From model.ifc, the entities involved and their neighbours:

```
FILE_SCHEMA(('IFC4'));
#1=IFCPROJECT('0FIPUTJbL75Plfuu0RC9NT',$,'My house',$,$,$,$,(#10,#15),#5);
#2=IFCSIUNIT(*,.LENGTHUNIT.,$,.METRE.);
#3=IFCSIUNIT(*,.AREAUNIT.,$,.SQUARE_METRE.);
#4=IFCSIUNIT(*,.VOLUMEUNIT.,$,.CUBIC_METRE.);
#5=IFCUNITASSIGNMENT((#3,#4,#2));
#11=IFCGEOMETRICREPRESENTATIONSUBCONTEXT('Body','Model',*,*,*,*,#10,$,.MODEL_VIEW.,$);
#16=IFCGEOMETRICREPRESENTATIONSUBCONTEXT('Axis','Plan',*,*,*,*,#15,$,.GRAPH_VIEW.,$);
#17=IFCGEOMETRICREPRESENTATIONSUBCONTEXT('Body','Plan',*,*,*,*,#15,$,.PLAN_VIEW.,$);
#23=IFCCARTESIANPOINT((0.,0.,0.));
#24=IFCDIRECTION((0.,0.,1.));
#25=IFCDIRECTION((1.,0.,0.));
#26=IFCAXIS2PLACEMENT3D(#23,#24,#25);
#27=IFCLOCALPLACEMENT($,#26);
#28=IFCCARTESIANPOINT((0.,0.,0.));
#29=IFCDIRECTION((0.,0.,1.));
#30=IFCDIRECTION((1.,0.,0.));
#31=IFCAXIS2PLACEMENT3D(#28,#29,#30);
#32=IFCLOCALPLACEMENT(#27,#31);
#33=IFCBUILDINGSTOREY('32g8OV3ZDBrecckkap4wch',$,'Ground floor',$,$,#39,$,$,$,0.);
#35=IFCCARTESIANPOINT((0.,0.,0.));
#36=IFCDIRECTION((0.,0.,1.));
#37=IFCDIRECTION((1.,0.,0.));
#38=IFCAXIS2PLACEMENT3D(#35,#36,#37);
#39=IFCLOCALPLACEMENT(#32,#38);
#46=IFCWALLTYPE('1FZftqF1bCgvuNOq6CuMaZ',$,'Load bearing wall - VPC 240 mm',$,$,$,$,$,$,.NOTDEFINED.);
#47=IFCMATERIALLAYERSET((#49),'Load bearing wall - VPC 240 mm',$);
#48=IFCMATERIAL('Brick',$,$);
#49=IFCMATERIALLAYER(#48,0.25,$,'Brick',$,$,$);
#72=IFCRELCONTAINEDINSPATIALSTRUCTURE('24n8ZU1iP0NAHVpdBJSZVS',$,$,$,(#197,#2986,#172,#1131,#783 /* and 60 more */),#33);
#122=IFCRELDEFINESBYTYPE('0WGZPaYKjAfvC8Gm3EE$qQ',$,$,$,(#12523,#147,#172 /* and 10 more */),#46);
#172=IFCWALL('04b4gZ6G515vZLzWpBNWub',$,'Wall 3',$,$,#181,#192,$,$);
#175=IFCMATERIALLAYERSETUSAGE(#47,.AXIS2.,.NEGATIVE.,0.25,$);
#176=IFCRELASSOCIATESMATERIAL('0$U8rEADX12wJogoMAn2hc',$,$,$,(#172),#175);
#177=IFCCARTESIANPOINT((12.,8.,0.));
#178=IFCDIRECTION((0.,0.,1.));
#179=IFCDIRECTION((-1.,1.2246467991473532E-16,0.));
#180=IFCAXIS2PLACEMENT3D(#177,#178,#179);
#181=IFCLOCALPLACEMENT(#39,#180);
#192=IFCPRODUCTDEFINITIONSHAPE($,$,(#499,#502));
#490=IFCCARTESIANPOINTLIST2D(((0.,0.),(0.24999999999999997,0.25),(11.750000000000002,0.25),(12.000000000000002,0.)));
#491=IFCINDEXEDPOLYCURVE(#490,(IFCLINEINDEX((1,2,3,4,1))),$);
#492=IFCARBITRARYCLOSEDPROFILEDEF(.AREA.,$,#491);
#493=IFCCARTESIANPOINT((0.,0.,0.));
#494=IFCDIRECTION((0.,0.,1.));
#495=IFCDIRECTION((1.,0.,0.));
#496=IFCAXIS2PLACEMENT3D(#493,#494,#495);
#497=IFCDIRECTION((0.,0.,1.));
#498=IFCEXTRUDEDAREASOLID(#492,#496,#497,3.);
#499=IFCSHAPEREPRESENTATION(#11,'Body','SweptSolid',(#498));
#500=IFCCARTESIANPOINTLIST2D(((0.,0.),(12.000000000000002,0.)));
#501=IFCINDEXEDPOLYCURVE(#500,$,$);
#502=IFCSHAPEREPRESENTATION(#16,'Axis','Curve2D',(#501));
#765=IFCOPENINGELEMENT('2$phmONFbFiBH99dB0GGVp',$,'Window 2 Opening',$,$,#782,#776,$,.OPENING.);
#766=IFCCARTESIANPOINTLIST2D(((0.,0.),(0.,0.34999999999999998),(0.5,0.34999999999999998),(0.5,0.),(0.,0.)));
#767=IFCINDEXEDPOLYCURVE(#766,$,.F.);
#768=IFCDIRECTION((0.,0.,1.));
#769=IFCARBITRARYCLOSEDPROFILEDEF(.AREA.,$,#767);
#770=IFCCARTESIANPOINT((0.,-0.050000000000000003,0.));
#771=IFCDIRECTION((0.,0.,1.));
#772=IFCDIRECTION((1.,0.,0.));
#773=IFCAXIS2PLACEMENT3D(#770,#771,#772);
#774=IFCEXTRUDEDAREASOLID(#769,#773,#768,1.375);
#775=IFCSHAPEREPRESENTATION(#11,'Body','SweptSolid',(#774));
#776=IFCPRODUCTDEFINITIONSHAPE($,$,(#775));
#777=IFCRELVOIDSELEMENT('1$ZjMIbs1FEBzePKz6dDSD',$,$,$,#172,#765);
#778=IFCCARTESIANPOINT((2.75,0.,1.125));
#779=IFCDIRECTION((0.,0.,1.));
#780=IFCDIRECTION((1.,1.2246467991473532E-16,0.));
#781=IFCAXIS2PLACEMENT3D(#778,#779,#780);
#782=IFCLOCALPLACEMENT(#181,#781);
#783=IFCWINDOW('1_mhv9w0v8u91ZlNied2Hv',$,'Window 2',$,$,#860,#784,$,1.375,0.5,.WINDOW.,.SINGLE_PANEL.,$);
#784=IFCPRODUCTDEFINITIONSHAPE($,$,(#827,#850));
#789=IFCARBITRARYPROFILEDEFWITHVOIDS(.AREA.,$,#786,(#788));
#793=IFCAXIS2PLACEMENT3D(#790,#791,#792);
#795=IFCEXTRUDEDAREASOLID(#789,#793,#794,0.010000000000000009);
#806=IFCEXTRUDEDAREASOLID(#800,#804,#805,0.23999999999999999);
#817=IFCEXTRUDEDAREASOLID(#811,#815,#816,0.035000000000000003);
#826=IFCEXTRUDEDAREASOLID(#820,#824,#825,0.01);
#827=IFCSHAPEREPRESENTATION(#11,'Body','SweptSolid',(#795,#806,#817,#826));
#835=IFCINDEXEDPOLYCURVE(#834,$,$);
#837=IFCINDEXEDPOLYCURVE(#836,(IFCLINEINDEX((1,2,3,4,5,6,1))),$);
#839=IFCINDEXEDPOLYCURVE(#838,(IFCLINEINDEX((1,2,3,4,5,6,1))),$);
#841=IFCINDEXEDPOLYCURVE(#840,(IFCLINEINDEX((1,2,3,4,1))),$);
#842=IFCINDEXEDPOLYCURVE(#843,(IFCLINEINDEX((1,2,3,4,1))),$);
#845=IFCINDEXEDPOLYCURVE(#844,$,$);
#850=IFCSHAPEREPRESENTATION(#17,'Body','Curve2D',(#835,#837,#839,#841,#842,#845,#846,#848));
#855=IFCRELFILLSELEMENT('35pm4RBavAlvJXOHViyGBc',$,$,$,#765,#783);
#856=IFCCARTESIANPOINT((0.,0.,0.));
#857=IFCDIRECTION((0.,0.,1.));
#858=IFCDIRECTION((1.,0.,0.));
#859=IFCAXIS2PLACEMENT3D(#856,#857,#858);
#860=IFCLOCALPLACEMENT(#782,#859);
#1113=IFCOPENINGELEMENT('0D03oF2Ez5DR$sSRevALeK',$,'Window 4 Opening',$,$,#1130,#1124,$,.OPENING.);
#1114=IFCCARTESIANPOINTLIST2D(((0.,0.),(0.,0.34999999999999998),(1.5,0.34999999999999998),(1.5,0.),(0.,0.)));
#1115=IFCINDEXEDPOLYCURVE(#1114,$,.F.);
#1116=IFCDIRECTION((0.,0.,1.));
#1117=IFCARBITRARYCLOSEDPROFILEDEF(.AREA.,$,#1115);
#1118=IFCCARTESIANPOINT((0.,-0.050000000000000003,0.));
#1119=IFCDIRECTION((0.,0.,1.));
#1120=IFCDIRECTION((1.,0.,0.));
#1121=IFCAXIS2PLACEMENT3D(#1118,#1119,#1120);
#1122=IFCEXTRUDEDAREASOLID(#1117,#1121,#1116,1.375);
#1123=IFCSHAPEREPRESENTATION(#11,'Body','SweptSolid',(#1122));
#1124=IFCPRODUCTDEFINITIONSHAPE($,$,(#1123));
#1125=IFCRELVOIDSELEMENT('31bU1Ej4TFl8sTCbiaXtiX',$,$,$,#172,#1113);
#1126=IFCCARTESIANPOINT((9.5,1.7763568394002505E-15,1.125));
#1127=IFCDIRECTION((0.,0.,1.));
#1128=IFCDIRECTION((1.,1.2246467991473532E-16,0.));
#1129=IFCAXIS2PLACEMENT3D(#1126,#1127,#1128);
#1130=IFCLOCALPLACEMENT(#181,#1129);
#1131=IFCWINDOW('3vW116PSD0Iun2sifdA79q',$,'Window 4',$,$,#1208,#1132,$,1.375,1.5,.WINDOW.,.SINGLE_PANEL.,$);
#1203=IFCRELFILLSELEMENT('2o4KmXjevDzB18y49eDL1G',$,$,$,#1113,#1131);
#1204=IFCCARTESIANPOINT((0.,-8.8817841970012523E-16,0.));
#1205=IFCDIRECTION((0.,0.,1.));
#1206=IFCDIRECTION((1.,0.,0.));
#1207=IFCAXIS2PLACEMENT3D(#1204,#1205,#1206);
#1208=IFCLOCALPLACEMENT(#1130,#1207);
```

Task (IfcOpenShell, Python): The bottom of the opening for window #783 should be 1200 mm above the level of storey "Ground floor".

```python
import numpy as np
import ifcopenshell
import ifcopenshell.api.geometry
import ifcopenshell.geom
import ifcopenshell.util.element
import ifcopenshell.util.placement
import ifcopenshell.util.shape
import ifcopenshell.util.unit

model = ifcopenshell.open("model.ifc")
unit_scale = ifcopenshell.util.unit.calculate_unit_scale(model)

window = model.by_guid("1_mhv9w0v8u91ZlNied2Hv")
opening = window.FillsVoids[0].RelatingOpeningElement
storey = ifcopenshell.util.element.get_container(window, ifc_class="IfcBuildingStorey")
level = ifcopenshell.util.placement.get_local_placement(storey.ObjectPlacement)[2, 3]

# The opening's origin need not be at the sill, so measure its lowest point.
shape = ifcopenshell.geom.create_shape(ifcopenshell.geom.settings(), opening)
bottom = ifcopenshell.util.shape.get_shape_bottom_elevation(shape, shape.geometry) / unit_scale
dz = level + 1.2 - bottom

shift = np.array([0.0, 0.0, dz])
# The window is placed relative to its opening, so it follows when the opening moves.
matrix = ifcopenshell.util.placement.get_local_placement(opening.ObjectPlacement)
matrix[:3, 3] += shift
ifcopenshell.api.geometry.edit_object_placement(
    model, product=opening, matrix=matrix, is_si=False, should_transform_children=True
)

print(f"moved by {dz * unit_scale:+.3f} m")

model.write("model_rev.ifc")
```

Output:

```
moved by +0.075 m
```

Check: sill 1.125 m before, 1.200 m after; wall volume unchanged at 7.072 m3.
